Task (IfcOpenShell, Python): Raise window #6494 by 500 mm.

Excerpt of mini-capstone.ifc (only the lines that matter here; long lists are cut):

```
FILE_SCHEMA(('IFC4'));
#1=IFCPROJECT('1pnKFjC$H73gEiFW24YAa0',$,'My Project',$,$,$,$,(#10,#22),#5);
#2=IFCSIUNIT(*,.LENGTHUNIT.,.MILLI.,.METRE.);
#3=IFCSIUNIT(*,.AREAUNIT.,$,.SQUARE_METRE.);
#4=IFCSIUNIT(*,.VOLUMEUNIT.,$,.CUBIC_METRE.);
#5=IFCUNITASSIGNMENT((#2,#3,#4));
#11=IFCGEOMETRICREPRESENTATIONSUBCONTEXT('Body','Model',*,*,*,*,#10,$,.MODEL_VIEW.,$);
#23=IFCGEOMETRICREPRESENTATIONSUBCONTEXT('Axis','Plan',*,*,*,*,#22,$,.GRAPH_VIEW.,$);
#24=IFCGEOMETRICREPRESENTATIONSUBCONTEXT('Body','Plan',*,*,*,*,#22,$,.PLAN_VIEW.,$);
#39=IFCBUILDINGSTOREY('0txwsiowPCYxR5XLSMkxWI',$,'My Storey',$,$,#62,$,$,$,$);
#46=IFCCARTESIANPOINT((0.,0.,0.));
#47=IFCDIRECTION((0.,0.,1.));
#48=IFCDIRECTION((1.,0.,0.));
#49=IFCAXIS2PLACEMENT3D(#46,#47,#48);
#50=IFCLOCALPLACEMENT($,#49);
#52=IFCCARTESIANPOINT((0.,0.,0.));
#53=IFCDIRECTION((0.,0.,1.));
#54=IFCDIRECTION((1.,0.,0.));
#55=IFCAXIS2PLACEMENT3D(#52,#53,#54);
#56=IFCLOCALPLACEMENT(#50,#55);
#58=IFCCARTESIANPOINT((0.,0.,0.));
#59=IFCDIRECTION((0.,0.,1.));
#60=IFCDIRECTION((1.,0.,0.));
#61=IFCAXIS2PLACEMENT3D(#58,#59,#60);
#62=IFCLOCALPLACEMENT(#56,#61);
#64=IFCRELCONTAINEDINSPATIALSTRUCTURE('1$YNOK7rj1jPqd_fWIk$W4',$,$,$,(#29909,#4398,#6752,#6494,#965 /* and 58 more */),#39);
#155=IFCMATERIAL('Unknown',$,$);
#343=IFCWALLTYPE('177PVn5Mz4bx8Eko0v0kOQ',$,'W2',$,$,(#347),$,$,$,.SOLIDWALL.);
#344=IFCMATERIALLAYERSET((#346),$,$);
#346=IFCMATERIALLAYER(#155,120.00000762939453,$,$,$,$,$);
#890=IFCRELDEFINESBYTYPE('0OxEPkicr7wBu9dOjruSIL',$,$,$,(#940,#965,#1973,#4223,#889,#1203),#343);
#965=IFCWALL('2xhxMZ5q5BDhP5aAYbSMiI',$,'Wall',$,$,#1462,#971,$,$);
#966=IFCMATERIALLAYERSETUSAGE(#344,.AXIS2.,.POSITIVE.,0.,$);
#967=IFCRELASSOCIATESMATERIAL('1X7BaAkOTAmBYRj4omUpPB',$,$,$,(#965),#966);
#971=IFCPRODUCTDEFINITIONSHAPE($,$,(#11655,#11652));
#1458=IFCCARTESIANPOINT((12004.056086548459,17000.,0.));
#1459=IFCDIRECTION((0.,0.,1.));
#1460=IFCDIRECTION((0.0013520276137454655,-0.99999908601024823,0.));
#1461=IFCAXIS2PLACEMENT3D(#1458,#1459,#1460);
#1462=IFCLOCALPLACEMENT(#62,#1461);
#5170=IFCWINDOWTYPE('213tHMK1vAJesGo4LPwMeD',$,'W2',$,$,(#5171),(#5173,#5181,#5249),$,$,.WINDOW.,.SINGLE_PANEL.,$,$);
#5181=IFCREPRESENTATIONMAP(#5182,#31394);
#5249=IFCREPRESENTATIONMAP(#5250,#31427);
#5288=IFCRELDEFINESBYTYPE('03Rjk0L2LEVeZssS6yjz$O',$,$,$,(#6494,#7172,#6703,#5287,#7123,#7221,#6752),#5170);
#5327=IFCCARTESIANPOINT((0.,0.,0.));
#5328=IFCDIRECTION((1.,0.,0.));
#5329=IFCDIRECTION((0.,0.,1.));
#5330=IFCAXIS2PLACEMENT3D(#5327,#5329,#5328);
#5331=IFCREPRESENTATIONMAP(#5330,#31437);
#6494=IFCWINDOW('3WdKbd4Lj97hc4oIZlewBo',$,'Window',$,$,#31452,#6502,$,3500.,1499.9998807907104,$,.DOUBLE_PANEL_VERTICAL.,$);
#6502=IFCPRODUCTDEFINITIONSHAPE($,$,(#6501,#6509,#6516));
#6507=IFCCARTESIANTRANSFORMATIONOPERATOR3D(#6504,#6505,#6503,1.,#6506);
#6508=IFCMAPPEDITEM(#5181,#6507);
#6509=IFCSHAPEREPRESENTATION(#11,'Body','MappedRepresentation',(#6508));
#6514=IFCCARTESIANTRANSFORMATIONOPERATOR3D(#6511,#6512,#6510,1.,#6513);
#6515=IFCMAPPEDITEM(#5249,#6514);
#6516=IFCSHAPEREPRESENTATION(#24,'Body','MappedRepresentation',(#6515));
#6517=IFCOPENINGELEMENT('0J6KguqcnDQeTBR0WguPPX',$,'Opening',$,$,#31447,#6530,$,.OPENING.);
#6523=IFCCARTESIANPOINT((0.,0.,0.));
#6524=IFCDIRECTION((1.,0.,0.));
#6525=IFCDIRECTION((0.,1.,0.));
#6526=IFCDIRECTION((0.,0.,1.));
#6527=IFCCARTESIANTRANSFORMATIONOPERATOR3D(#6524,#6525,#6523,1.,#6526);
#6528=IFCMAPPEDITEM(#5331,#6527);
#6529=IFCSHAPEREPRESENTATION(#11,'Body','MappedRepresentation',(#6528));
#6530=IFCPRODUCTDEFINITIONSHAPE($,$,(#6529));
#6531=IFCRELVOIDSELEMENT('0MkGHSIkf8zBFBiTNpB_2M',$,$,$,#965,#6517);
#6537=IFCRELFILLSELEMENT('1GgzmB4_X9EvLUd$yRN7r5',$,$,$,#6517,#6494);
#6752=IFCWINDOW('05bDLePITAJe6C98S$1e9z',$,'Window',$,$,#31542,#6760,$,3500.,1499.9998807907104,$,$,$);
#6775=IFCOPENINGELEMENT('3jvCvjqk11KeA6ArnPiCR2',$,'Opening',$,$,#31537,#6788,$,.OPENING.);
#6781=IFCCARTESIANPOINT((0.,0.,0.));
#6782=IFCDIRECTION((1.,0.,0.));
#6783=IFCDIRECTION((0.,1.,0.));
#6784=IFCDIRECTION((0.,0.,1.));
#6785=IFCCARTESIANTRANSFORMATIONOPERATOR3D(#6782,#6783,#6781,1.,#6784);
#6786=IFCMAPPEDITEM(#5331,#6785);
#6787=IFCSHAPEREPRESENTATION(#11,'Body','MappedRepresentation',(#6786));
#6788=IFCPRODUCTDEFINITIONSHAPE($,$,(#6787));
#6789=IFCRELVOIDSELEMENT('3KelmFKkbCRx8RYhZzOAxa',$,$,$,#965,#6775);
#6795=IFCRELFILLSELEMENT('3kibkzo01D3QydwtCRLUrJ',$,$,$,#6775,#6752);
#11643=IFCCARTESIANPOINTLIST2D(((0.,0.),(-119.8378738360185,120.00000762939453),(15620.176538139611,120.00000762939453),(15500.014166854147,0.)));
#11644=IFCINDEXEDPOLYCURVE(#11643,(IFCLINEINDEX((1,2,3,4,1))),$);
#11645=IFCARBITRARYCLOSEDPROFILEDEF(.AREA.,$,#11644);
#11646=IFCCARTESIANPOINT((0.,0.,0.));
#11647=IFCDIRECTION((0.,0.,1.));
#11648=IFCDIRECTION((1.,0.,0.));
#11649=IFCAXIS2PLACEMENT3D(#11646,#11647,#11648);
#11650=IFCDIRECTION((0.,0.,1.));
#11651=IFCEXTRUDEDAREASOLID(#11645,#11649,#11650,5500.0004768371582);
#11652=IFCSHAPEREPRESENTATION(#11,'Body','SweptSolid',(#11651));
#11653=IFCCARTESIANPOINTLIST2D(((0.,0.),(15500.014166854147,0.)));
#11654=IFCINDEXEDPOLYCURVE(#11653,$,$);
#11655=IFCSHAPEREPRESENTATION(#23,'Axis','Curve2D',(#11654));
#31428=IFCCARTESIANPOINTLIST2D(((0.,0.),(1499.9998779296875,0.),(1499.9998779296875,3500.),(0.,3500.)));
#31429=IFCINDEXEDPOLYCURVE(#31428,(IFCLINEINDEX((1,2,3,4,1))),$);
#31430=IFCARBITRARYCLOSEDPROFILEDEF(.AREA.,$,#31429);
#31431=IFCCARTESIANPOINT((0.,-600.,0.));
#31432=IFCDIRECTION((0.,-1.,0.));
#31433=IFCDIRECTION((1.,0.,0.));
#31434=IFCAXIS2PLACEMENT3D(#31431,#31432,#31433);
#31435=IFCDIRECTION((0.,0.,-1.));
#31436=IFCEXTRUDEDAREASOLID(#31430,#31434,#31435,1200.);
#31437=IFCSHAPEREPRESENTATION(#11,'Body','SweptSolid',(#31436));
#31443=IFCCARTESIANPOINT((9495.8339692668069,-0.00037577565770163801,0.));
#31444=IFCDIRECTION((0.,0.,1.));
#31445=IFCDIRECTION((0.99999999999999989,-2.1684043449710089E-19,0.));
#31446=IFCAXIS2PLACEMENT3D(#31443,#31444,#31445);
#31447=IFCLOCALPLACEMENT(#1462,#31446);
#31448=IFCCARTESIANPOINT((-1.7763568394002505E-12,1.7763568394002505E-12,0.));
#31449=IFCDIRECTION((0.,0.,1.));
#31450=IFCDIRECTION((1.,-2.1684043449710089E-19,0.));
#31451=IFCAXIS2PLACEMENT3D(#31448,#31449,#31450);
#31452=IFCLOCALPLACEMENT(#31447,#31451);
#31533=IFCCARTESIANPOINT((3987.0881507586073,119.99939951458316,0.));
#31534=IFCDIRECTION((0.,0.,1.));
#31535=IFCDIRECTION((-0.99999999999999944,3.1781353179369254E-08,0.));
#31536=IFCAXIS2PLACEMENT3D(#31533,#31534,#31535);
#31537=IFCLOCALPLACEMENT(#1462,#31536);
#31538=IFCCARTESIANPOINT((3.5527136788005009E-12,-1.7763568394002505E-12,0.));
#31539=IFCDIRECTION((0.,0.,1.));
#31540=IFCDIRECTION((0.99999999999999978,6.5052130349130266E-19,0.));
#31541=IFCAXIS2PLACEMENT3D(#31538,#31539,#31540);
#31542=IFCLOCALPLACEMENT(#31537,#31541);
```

```python
import numpy as np
import ifcopenshell
import ifcopenshell.api.geometry
import ifcopenshell.util.placement
import ifcopenshell.util.unit

model = ifcopenshell.open("mini-capstone.ifc")
unit_scale = ifcopenshell.util.unit.calculate_unit_scale(model)

window = model.by_guid("3WdKbd4Lj97hc4oIZlewBo")
opening = window.FillsVoids[0].RelatingOpeningElement
dz = 0.5 / unit_scale

shift = np.array([0.0, 0.0, dz])
# The window is placed relative to its opening, so it follows when the opening moves.
matrix = ifcopenshell.util.placement.get_local_placement(opening.ObjectPlacement)
matrix[:3, 3] += shift
ifcopenshell.api.geometry.edit_object_placement(
    model, product=opening, matrix=matrix, is_si=False, should_transform_children=True
)

print(f"moved by {dz * unit_scale:+.3f} m")

model.write("mini-capstone-out.ifc")
```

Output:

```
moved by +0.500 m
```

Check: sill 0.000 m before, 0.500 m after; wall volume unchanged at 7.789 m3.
